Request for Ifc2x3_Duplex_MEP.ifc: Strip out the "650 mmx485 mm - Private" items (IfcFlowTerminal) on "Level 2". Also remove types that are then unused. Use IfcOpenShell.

First a look at what the model holds.

```python
import ifcopenshell
import ifcopenshell.util.element

model = ifcopenshell.open("Ifc2x3_Duplex_MEP.ifc")
print(model.schema)
storey = next(s for s in model.by_type("IfcBuildingStorey") if s.Name == "Level 2")
terminals = [e for e in ifcopenshell.util.element.get_decomposition(storey) if e.is_a("IfcFlowTerminal")]
seen = {}
for e in terminals:
    element_type = ifcopenshell.util.element.get_type(e)
    name = element_type.Name if element_type not in (None, e) else None
    seen[name] = seen.get(name, 0) + 1
for name, count in sorted(seen.items(), key=str):
    print(count, "x", name)
```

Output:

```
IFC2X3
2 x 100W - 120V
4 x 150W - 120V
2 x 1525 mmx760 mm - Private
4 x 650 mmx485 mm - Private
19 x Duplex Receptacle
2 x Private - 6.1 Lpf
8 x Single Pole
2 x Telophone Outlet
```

```python
import ifcopenshell
import ifcopenshell.api.root
import ifcopenshell.util.element

model = ifcopenshell.open("Ifc2x3_Duplex_MEP.ifc")

storey = next(s for s in model.by_type("IfcBuildingStorey") if s.Name == "Level 2")
terminals = [e for e in ifcopenshell.util.element.get_decomposition(storey) if e.is_a("IfcFlowTerminal")]
targets = [e for e in terminals if (t := ifcopenshell.util.element.get_type(e)) not in (None, e) and t.Name == "650 mmx485 mm - Private"]
types = {ifcopenshell.util.element.get_type(e) for e in targets} - {None, *targets}

for e in targets:
    ifcopenshell.api.root.remove_product(model, product=e)
print(len(targets), "removed")

unused = [t for t in types if not ifcopenshell.util.element.get_types(t)]
for t in unused:
    ifcopenshell.api.root.remove_product(model, product=t)
print(len(unused), "unused types removed")

model.write("Ifc2x3_Duplex_MEP_edited.ifc")
```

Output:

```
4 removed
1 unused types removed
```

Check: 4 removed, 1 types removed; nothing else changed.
